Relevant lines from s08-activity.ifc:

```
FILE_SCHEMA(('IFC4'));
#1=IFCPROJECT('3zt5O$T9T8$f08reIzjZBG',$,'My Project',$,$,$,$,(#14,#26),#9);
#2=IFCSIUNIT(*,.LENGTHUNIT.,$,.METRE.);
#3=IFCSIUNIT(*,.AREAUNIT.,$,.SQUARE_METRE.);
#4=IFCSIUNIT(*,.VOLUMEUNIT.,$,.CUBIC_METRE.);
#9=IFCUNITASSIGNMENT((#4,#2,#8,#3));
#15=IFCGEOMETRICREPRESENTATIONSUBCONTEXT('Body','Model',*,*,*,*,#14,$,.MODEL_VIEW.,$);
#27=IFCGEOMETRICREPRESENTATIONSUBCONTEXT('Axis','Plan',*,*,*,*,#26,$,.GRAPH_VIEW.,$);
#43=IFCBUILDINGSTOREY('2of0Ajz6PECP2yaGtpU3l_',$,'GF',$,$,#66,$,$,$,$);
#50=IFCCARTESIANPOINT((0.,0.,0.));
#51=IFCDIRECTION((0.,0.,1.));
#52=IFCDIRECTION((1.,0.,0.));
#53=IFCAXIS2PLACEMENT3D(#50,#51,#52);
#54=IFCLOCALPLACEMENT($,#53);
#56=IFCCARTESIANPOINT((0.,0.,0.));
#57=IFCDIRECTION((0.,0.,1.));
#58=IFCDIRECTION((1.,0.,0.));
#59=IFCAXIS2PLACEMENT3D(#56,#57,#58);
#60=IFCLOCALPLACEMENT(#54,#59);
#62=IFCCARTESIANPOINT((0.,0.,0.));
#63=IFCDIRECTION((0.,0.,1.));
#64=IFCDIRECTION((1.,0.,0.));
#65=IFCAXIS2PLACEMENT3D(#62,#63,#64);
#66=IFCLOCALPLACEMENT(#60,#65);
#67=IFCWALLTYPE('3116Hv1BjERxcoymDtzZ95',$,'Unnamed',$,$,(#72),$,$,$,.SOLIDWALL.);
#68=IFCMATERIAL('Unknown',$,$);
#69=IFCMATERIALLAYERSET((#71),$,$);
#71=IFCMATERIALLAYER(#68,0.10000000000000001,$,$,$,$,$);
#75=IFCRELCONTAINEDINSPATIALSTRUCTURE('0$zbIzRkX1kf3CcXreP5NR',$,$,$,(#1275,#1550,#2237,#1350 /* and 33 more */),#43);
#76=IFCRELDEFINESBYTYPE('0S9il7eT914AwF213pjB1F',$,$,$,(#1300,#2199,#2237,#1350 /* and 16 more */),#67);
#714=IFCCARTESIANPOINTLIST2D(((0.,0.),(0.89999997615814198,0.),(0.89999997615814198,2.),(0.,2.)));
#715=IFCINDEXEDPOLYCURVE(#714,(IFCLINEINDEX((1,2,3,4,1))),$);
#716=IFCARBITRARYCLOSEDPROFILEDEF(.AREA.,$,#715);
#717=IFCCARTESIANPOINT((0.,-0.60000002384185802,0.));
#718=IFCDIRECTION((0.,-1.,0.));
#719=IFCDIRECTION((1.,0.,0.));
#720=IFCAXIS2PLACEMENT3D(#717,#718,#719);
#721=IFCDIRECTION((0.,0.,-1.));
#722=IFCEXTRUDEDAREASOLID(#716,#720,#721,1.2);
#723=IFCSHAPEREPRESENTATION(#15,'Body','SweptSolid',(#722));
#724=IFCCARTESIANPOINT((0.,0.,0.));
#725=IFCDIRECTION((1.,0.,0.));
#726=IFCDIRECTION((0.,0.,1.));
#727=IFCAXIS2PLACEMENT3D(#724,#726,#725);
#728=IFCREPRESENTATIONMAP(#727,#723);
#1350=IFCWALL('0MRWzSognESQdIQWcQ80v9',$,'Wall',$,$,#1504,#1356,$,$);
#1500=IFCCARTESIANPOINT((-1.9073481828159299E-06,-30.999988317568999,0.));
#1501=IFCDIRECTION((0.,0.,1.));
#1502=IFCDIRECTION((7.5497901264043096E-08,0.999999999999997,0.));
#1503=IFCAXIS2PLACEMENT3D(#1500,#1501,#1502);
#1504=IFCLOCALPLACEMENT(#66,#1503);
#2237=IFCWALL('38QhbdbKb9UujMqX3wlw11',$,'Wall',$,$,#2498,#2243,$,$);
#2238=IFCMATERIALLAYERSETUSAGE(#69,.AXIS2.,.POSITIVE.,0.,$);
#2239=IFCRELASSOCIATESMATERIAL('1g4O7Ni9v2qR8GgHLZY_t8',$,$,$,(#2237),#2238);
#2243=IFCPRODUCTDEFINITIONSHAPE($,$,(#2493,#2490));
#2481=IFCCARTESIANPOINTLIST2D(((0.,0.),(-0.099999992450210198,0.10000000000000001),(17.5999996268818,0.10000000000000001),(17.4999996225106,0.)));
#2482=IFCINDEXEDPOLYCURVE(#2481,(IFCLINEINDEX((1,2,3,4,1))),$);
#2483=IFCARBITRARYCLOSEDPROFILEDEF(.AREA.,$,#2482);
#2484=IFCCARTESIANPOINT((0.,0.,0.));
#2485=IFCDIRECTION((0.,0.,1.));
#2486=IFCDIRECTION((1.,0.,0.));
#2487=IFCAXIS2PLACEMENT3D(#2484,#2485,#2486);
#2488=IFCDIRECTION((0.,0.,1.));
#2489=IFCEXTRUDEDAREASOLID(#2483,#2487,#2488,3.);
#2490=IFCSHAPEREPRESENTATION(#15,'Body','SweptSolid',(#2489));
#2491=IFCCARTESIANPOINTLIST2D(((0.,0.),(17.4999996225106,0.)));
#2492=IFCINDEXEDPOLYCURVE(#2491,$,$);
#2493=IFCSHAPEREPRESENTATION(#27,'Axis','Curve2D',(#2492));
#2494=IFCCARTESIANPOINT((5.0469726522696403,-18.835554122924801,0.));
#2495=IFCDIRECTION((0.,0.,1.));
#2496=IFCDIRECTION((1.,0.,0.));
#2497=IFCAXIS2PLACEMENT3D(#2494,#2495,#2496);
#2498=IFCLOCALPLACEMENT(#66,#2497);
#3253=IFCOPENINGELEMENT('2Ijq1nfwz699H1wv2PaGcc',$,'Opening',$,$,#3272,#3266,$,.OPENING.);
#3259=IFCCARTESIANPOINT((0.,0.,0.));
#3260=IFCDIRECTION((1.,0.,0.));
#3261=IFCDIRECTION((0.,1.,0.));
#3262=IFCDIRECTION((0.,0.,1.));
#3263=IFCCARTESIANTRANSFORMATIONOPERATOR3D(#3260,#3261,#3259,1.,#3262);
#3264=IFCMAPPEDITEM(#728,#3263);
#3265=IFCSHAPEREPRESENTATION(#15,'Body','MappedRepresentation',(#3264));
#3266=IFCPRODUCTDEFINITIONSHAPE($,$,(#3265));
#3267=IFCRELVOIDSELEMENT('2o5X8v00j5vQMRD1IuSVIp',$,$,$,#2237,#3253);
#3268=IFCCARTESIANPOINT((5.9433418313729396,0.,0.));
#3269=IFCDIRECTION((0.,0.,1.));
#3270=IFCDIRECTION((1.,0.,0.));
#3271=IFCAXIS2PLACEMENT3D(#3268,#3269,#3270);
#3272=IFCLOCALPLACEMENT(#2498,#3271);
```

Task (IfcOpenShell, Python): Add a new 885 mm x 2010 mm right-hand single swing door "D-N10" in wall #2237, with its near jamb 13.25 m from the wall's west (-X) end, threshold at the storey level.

```python
import numpy as np
import ifcopenshell
import ifcopenshell.api.feature
import ifcopenshell.api.geometry
import ifcopenshell.api.root
import ifcopenshell.api.spatial
import ifcopenshell.geom
import ifcopenshell.util.element
import ifcopenshell.util.placement
import ifcopenshell.util.representation
import ifcopenshell.util.shape
import ifcopenshell.util.unit

model = ifcopenshell.open("s08-activity.ifc")
unit_scale = ifcopenshell.util.unit.calculate_unit_scale(model)
settings = ifcopenshell.geom.settings()


def volume(element):
    """Net volume in cubic metres, openings subtracted."""
    shape = ifcopenshell.geom.create_shape(settings, element)
    return ifcopenshell.util.shape.get_volume(shape.geometry)


wall = model.by_guid("38QhbdbKb9UujMqX3wlw11")
storey = ifcopenshell.util.element.get_container(wall, ifc_class="IfcBuildingStorey")
context = ifcopenshell.util.representation.get_context(model, "Model", "Body", "MODEL_VIEW")
before = volume(wall)

width, height, from_end, sill = 0.885, 2.01, 13.25, 0.0  # metres

# The wall runs along its own X axis, and the end named is its -X end.
wall_shape = ifcopenshell.geom.create_shape(settings, wall)
x, y, z = ifcopenshell.util.shape.get_vertices(wall_shape.geometry).T
start = x.min() + from_end
face, thickness = float(y.min()), float(y.max() - y.min())
wall_matrix = ifcopenshell.util.placement.get_local_placement(wall.ObjectPlacement)
level = ifcopenshell.util.placement.get_local_placement(storey.ObjectPlacement)[2, 3]


def in_wall(x, y):
    """Placement at x, y metres in the wall's axes, at sill height."""
    matrix = wall_matrix.copy()
    matrix[:, 3] = wall_matrix @ np.array([x / unit_scale, y / unit_scale, 0.0, 1.0])
    matrix[2, 3] = level + sill / unit_scale
    return matrix


# Opening: a box that overshoots both wall faces by 50 mm.
opening = ifcopenshell.api.root.create_entity(model, ifc_class="IfcOpeningElement", predefined_type="OPENING")
box = ifcopenshell.api.geometry.add_wall_representation(
    model, context=context, length=width, height=height, thickness=thickness + 0.1
)
ifcopenshell.api.geometry.assign_representation(model, product=opening, representation=box)
ifcopenshell.api.geometry.edit_object_placement(model, product=opening, matrix=in_wall(start, face - 0.05), is_si=False)
ifcopenshell.api.feature.add_feature(model, feature=opening, element=wall)

door = ifcopenshell.api.root.create_entity(model, ifc_class="IfcDoor", name="D-N10", predefined_type="DOOR")
door.OverallWidth, door.OverallHeight = width / unit_scale, height / unit_scale
door.OperationType = "SINGLE_SWING_RIGHT"
body = ifcopenshell.api.geometry.add_door_representation(
    model,
    context=context,
    overall_width=door.OverallWidth,
    overall_height=door.OverallHeight,
    operation_type="SINGLE_SWING_RIGHT",
    lining_properties={"LiningDepth": thickness / unit_scale, "ThresholdDepth": thickness / unit_scale},
)
ifcopenshell.api.geometry.assign_representation(model, product=door, representation=body)
ifcopenshell.api.spatial.assign_container(model, products=[door], relating_structure=storey)
ifcopenshell.api.feature.add_filling(model, opening=opening, element=door)

# The lining spans the wall, so the door starts at the wall face.
ifcopenshell.api.geometry.edit_object_placement(model, product=door, matrix=in_wall(start, face), is_si=False)

after = volume(wall)

print(f"wall volume {before:.3f} -> {after:.3f} m3")

model.write("s08-activity_updated.ifc")
```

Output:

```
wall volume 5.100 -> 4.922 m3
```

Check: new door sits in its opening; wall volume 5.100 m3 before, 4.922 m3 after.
